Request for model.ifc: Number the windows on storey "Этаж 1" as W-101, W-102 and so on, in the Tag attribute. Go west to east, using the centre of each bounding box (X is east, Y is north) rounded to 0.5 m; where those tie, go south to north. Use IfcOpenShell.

First a look at what the model holds.

```python
import ifcopenshell
import ifcopenshell.util.element
import ifcopenshell.util.placement

model = ifcopenshell.open("model.ifc")
print(model.schema)
storey = next(s for s in model.by_type("IfcBuildingStorey") if s.Name == "Этаж 1")
windows = [e for e in ifcopenshell.util.element.get_decomposition(storey) if e.is_a("IfcWindow")]
for e in sorted(windows, key=lambda e: e.id()):
    origin = ifcopenshell.util.placement.get_local_placement(e.ObjectPlacement)[:3, 3]
    print(e.id(), e.Tag, e.Name, origin.round(2) + 0.0, sep=" | ")
```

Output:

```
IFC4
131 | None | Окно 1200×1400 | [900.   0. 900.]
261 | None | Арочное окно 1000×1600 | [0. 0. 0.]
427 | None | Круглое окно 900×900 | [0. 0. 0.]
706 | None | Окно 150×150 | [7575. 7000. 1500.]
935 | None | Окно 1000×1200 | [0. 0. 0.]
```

```python
import ifcopenshell
import ifcopenshell.geom
import ifcopenshell.util.element
import ifcopenshell.util.shape

model = ifcopenshell.open("model.ifc")
settings = ifcopenshell.geom.settings()
settings.set("use-world-coords", True)


def centre(element):
    shape = ifcopenshell.geom.create_shape(settings, element)
    return ifcopenshell.util.shape.get_bbox_centroid(shape.geometry)


storey = next(s for s in model.by_type("IfcBuildingStorey") if s.Name == "Этаж 1")
windows = [e for e in ifcopenshell.util.element.get_decomposition(storey) if e.is_a("IfcWindow")]

# Insertion points can sit at a corner or the storey origin, so sort by the geometry (in metres).
centres = {e: centre(e) for e in windows}
windows.sort(key=lambda e: (round(centres[e][0] / 0.5), centres[e][1]))

for i, e in enumerate(windows, start=1):
    number = f"W-1{i:02d}"
    e.Tag = number
    print(e.id(), number)

model.write("model_rev.ifc")
```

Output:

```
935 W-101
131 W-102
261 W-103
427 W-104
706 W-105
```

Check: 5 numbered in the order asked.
